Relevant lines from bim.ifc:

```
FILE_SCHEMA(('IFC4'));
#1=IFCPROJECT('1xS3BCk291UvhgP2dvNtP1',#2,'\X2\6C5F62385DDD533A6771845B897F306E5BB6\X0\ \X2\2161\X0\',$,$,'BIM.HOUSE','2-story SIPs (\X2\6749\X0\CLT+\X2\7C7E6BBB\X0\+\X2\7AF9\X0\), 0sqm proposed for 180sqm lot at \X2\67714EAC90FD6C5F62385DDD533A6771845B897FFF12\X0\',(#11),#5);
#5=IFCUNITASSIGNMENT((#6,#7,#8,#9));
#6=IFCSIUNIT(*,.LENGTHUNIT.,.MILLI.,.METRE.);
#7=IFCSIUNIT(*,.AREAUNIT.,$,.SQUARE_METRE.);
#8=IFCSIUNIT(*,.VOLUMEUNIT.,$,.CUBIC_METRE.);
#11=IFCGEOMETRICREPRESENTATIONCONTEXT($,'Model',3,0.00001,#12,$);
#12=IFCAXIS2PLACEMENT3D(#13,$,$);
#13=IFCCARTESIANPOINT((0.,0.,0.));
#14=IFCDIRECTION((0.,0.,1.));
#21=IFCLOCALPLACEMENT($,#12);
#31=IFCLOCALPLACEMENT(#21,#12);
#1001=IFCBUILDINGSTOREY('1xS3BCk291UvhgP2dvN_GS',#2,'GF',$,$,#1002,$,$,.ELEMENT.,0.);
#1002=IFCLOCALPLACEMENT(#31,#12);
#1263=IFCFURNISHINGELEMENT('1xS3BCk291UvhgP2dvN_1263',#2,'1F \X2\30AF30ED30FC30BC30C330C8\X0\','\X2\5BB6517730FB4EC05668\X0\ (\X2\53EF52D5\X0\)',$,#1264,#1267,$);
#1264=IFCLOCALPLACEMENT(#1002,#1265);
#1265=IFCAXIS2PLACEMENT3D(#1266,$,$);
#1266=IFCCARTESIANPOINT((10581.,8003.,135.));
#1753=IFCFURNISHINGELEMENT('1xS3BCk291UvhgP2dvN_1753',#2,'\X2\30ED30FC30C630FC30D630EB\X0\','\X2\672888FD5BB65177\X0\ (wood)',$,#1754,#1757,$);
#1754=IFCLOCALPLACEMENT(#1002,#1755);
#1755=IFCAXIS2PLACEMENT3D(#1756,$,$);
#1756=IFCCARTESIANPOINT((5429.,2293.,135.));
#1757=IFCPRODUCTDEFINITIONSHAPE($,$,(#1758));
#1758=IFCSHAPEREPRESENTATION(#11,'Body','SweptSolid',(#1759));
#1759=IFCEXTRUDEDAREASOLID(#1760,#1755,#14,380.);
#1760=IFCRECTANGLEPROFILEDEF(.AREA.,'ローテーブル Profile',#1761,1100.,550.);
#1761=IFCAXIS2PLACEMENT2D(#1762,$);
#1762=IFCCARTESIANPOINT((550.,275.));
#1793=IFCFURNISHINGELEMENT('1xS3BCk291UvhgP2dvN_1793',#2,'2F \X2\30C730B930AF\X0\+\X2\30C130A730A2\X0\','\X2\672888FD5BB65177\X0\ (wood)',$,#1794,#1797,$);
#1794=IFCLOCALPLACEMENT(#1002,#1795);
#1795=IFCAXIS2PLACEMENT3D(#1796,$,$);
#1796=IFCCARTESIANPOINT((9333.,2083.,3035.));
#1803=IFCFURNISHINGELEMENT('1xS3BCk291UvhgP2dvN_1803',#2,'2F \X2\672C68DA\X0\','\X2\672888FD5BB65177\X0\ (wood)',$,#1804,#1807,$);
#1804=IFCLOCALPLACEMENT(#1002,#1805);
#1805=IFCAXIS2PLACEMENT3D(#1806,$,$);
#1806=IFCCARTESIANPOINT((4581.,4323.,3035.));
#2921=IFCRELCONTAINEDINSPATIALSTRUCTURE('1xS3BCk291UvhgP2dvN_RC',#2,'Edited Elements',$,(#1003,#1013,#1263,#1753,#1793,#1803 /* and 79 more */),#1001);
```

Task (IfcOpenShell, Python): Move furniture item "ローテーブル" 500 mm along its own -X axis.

```python
import ifcopenshell
import ifcopenshell.api.geometry
import ifcopenshell.util.placement

model = ifcopenshell.open("bim.ifc")

item = model.by_id(1753)
matrix = ifcopenshell.util.placement.get_local_placement(item.ObjectPlacement)
matrix[:3, 3] -= matrix[:3, 0] * 500.0
ifcopenshell.api.geometry.edit_object_placement(model, product=item, matrix=matrix, is_si=False)

print(ifcopenshell.util.placement.get_local_placement(item.ObjectPlacement).round(3) + 0.0)

model.write("bim_rev.ifc")
```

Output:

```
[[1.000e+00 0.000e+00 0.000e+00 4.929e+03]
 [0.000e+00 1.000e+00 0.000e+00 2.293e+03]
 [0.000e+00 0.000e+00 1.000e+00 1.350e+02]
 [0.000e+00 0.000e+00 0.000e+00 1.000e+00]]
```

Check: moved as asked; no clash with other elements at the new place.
